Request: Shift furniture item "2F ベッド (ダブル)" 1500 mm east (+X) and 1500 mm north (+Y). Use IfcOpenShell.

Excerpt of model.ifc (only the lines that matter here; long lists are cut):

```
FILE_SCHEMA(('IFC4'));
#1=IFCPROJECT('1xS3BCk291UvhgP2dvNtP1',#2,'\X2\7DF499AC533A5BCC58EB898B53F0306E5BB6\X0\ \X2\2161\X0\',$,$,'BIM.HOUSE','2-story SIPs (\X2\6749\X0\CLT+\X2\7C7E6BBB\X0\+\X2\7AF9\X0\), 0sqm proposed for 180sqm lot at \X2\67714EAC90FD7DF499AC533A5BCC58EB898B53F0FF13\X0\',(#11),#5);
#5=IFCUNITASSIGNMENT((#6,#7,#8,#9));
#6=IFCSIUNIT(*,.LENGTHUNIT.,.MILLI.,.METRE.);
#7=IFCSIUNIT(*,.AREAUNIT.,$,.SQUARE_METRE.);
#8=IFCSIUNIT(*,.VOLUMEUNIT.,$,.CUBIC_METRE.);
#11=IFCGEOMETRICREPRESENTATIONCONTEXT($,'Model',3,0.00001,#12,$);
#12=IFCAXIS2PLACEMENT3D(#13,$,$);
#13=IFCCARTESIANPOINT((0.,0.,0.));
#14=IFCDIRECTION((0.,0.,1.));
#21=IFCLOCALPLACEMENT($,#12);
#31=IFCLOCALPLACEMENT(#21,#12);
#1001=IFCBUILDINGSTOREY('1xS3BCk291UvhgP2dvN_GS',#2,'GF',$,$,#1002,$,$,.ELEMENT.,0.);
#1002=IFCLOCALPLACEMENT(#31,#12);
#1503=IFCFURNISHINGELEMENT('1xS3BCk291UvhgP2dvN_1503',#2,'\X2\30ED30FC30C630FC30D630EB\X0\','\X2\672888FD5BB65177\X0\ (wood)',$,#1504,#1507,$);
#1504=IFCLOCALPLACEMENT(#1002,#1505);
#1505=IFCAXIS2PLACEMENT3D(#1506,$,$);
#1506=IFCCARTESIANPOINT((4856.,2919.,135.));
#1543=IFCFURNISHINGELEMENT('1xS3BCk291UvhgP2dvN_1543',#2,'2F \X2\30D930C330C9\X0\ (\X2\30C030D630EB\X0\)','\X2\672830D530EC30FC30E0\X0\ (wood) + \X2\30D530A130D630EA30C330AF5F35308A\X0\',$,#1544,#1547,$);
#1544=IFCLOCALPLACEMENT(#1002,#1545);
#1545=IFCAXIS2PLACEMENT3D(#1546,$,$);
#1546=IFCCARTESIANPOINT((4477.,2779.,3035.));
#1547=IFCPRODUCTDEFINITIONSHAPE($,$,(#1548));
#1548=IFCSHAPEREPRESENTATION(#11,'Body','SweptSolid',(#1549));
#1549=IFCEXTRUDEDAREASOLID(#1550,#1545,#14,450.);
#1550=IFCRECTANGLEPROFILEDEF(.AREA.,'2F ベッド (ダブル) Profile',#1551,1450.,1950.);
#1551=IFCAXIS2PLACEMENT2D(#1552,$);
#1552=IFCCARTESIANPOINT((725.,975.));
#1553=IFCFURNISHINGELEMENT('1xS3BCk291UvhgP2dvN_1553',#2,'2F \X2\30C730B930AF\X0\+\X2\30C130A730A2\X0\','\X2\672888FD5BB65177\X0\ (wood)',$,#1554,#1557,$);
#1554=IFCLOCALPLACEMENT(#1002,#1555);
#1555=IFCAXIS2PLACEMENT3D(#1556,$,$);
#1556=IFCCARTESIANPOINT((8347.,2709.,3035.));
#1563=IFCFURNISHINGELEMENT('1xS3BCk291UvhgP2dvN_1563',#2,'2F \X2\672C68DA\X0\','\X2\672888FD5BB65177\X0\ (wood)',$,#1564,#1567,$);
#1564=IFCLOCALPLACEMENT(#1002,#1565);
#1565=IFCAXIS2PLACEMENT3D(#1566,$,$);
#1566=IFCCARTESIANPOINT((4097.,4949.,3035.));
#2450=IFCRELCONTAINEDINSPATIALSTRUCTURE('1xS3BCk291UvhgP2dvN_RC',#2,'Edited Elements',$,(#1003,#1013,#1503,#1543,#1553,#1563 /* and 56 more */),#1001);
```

```python
import ifcopenshell
import ifcopenshell.api.geometry
import ifcopenshell.util.placement

model = ifcopenshell.open("model.ifc")

item = model.by_id(1543)
matrix = ifcopenshell.util.placement.get_local_placement(item.ObjectPlacement)
matrix[0, 3] += 1500.0
matrix[1, 3] += 1500.0
ifcopenshell.api.geometry.edit_object_placement(model, product=item, matrix=matrix, is_si=False)

print(ifcopenshell.util.placement.get_local_placement(item.ObjectPlacement).round(3) + 0.0)

model.write("model-out.ifc")
```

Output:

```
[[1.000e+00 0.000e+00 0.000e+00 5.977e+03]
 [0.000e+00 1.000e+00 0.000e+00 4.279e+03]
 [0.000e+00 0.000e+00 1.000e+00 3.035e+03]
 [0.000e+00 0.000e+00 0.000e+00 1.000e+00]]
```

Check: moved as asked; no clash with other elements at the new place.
